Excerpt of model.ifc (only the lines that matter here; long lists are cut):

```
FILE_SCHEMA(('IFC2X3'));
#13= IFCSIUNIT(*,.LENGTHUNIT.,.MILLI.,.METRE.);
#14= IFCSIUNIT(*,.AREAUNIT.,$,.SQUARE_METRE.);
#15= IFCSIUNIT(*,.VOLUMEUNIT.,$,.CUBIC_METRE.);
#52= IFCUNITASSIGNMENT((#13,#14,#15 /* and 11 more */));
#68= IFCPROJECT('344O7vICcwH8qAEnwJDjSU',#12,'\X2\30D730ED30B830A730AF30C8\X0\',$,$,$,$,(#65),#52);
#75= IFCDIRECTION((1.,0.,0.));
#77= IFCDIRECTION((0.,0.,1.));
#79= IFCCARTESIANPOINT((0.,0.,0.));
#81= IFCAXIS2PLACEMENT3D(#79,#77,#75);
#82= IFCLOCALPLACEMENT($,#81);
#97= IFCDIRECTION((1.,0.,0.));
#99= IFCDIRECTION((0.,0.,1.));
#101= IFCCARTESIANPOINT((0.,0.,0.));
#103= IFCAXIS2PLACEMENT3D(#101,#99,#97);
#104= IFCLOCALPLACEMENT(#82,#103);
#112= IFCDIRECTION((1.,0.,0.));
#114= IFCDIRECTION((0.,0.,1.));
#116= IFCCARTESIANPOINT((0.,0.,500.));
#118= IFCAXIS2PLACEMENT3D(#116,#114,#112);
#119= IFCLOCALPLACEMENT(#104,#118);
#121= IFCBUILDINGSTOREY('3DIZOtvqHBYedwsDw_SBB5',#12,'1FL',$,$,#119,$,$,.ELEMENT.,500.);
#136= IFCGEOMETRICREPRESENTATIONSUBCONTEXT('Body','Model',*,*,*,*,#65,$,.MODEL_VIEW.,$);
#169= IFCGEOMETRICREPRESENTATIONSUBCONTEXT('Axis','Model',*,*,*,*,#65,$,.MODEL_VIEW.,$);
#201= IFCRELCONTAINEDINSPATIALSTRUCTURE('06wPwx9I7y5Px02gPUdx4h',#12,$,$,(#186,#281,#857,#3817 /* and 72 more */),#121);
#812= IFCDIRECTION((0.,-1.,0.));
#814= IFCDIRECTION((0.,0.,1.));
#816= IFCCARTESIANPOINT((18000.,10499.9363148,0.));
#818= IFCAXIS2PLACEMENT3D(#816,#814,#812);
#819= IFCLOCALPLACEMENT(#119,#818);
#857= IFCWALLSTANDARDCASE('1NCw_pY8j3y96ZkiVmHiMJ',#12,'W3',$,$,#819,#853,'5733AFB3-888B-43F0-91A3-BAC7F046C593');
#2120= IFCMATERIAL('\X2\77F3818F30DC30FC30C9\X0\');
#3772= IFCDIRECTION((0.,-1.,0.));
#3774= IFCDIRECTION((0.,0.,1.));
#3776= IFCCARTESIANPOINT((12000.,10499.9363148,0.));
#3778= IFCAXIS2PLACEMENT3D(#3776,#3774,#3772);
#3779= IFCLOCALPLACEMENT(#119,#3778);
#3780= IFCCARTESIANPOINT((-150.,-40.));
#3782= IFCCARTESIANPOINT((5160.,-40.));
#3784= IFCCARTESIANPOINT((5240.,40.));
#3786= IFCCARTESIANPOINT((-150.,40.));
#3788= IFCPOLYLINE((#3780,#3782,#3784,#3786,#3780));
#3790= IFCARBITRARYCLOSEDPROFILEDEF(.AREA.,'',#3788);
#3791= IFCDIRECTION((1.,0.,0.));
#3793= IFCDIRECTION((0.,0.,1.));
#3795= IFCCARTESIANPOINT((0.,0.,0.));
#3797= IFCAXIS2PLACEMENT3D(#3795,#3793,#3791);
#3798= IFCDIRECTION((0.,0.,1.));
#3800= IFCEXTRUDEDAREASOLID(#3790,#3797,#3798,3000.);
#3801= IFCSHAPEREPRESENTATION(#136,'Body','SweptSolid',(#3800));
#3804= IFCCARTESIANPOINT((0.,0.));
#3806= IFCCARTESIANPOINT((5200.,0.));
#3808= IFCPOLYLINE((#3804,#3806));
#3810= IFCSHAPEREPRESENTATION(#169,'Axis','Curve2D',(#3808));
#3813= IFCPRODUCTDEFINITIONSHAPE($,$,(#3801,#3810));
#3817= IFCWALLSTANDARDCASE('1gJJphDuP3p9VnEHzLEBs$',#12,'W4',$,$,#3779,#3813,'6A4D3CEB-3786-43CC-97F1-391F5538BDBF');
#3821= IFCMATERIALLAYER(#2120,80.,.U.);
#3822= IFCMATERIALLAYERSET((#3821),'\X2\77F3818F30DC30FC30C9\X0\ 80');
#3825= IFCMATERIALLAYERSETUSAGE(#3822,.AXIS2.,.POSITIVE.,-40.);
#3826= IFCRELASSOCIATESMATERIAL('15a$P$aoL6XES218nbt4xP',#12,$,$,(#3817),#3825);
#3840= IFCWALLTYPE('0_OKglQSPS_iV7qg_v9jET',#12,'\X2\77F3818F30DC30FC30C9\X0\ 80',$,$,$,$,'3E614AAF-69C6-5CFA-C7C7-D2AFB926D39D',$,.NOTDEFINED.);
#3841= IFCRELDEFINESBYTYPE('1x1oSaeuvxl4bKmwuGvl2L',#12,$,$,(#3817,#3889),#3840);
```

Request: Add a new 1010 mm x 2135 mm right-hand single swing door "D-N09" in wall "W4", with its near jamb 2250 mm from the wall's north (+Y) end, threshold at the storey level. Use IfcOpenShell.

```python
import numpy as np
import ifcopenshell
import ifcopenshell.api.feature
import ifcopenshell.api.geometry
import ifcopenshell.api.root
import ifcopenshell.api.spatial
import ifcopenshell.api.type
import ifcopenshell.geom
import ifcopenshell.util.element
import ifcopenshell.util.placement
import ifcopenshell.util.representation
import ifcopenshell.util.shape
import ifcopenshell.util.unit

model = ifcopenshell.open("model.ifc")
unit_scale = ifcopenshell.util.unit.calculate_unit_scale(model)
settings = ifcopenshell.geom.settings()


def volume(element):
    """Net volume in cubic metres, openings subtracted."""
    shape = ifcopenshell.geom.create_shape(settings, element)
    return ifcopenshell.util.shape.get_volume(shape.geometry)


wall = model.by_id(3817)
storey = ifcopenshell.util.element.get_container(wall, ifc_class="IfcBuildingStorey")
context = ifcopenshell.util.representation.get_context(model, "Model", "Body", "MODEL_VIEW")
before = volume(wall)

width, height, from_end, sill = 1.01, 2.135, 2.25, 0.0  # metres

# The wall runs along its own X axis, and the end named is its -X end.
wall_shape = ifcopenshell.geom.create_shape(settings, wall)
x, y, z = ifcopenshell.util.shape.get_vertices(wall_shape.geometry).T
start = x.min() + from_end
face, thickness = float(y.min()), float(y.max() - y.min())
wall_matrix = ifcopenshell.util.placement.get_local_placement(wall.ObjectPlacement)
level = ifcopenshell.util.placement.get_local_placement(storey.ObjectPlacement)[2, 3]


def in_wall(x, y):
    """Placement at x, y metres in the wall's axes, at sill height."""
    matrix = wall_matrix.copy()
    matrix[:, 3] = wall_matrix @ np.array([x / unit_scale, y / unit_scale, 0.0, 1.0])
    matrix[2, 3] = level + sill / unit_scale
    return matrix


# Opening: a box that overshoots both wall faces by 50 mm.
opening = ifcopenshell.api.root.create_entity(model, ifc_class="IfcOpeningElement")
box = ifcopenshell.api.geometry.add_wall_representation(
    model, context=context, length=width, height=height, thickness=thickness + 0.1
)
ifcopenshell.api.geometry.assign_representation(model, product=opening, representation=box)
ifcopenshell.api.geometry.edit_object_placement(model, product=opening, matrix=in_wall(start, face - 0.05), is_si=False)
ifcopenshell.api.feature.add_feature(model, feature=opening, element=wall)

door = ifcopenshell.api.root.create_entity(model, ifc_class="IfcDoor", name="D-N09")
door.OverallWidth, door.OverallHeight = width / unit_scale, height / unit_scale
body = ifcopenshell.api.geometry.add_door_representation(
    model,
    context=context,
    overall_width=door.OverallWidth,
    overall_height=door.OverallHeight,
    operation_type="SINGLE_SWING_RIGHT",
    lining_properties={"LiningDepth": thickness / unit_scale, "ThresholdDepth": thickness / unit_scale},
)
ifcopenshell.api.geometry.assign_representation(model, product=door, representation=body)
ifcopenshell.api.spatial.assign_container(model, products=[door], relating_structure=storey)
fills = ifcopenshell.api.feature.add_filling(model, opening=opening, element=door)
fills.OwnerHistory = door.OwnerHistory  # required in IFC2X3

# IFC2X3 keeps the operation on the door style.
style = ifcopenshell.api.root.create_entity(model, ifc_class="IfcDoorStyle", name="D-N09")
style.OperationType, style.ConstructionType = "SINGLE_SWING_RIGHT", "NOTDEFINED"
style.ParameterTakesPrecedence = style.Sizeable = False
ifcopenshell.api.type.assign_type(model, related_objects=[door], relating_type=style)

# The lining spans the wall, so the door starts at the wall face.
ifcopenshell.api.geometry.edit_object_placement(model, product=door, matrix=in_wall(start, face), is_si=False)

after = volume(wall)

print(f"wall volume {before:.3f} -> {after:.3f} m3")

model.write("model_v2.ifc")
```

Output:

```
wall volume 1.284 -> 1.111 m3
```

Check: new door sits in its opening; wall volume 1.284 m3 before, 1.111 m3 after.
